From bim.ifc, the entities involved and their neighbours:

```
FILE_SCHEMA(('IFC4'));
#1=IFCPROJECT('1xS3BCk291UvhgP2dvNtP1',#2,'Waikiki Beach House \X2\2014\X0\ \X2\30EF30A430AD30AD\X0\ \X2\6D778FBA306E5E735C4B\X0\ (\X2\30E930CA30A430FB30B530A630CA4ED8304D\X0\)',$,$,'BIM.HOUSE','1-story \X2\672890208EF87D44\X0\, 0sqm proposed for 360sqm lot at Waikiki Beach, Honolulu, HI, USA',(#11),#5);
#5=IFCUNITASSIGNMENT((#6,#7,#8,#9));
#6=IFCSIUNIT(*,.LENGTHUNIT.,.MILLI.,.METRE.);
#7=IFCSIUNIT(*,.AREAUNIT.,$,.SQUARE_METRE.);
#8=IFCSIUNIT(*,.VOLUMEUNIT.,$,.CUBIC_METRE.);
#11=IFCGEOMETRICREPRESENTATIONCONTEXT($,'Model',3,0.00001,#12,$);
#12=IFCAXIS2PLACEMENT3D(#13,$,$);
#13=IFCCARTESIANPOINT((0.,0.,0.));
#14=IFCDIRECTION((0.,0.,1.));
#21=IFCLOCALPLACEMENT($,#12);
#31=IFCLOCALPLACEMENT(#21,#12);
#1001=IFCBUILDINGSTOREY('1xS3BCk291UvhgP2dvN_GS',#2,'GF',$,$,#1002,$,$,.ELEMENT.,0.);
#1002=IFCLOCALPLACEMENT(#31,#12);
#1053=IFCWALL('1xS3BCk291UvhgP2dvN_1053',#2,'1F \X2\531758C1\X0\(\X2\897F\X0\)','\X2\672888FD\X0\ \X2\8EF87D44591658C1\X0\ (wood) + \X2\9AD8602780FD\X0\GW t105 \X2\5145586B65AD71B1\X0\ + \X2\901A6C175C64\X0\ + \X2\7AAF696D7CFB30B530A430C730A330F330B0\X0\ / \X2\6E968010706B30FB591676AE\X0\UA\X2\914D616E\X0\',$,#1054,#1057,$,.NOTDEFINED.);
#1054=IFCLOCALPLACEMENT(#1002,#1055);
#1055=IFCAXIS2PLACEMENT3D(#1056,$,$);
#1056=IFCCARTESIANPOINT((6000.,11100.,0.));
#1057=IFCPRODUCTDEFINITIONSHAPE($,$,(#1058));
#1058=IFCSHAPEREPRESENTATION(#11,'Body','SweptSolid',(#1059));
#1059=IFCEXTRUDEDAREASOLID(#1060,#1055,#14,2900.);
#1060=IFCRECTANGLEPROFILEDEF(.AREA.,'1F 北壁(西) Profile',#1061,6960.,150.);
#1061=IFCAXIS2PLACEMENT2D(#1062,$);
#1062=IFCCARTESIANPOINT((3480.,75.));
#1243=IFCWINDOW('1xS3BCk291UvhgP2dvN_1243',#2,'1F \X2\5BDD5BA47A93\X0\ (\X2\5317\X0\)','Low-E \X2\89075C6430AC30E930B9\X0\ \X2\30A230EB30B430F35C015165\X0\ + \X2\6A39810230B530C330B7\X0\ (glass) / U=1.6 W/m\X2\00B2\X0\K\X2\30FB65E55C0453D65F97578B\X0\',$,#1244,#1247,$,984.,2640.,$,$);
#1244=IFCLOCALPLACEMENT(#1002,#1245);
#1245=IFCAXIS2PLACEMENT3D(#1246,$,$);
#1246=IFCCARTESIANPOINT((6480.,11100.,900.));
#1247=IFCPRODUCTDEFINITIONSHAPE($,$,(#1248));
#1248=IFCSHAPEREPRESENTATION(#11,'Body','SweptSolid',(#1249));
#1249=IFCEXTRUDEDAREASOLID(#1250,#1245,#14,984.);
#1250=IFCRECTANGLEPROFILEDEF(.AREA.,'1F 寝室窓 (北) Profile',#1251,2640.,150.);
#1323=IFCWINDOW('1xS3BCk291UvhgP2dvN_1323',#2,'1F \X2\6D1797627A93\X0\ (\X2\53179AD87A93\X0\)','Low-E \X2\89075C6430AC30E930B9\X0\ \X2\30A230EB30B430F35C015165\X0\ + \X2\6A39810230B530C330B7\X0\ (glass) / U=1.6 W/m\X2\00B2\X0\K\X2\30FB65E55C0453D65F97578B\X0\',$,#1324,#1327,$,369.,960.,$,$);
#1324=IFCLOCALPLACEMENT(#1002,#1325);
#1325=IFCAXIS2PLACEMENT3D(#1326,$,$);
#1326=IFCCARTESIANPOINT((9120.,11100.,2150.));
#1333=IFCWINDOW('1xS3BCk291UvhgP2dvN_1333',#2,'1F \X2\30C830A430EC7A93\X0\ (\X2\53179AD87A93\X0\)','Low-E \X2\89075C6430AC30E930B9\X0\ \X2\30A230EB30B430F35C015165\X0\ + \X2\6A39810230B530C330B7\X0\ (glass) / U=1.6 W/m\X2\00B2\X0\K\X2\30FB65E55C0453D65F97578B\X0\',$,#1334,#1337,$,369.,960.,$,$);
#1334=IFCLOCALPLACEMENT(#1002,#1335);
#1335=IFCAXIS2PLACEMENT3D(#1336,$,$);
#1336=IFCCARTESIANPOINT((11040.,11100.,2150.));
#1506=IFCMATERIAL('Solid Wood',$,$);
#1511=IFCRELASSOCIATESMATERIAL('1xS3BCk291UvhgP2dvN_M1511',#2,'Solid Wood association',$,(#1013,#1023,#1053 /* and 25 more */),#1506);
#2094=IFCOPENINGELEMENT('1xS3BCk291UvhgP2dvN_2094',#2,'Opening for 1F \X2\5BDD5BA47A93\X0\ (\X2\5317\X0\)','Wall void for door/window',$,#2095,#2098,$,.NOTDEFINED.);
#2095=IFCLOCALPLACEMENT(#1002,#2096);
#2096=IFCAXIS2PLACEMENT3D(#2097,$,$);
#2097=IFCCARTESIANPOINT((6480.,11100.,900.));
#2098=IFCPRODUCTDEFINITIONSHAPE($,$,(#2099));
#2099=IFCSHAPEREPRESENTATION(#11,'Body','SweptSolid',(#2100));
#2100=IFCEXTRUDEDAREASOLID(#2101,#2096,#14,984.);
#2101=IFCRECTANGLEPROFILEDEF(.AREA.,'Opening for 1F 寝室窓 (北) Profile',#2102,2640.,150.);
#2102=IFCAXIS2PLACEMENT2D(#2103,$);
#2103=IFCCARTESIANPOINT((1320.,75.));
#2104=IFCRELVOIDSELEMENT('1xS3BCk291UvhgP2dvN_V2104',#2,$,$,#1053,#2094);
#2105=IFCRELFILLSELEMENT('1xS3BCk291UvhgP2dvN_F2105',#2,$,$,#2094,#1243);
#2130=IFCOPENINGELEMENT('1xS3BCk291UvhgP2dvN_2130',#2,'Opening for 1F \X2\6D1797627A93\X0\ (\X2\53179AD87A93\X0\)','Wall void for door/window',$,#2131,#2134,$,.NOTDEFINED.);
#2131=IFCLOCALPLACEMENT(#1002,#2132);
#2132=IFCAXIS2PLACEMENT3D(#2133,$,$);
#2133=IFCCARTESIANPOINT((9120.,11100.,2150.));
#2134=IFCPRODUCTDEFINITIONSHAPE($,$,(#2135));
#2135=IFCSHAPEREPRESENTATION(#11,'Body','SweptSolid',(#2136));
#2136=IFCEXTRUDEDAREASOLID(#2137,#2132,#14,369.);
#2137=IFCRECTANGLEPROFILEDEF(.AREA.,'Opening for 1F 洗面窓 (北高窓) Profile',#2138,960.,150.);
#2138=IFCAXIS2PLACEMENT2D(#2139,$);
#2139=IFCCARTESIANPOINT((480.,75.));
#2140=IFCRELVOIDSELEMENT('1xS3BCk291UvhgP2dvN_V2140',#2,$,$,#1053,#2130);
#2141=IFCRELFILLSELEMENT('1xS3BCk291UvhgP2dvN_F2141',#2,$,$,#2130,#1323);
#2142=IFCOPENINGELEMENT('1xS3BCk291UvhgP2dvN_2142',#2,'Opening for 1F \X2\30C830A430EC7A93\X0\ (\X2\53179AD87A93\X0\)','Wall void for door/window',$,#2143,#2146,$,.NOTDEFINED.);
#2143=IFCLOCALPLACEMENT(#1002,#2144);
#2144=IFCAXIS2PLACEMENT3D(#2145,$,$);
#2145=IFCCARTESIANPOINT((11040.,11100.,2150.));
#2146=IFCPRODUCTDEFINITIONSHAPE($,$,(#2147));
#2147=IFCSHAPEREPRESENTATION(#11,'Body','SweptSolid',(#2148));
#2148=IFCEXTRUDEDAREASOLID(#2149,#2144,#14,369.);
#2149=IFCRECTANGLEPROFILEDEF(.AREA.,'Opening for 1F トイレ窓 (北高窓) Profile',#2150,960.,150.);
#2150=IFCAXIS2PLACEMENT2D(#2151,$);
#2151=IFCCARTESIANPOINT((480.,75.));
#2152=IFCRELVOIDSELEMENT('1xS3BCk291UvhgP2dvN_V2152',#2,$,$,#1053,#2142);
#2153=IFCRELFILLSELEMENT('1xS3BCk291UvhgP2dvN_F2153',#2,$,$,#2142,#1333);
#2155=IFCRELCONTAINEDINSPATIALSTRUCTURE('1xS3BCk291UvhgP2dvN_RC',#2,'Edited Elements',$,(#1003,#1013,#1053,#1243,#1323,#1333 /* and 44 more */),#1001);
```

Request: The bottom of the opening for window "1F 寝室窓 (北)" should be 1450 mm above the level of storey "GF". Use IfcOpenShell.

```python
import numpy as np
import ifcopenshell
import ifcopenshell.api.geometry
import ifcopenshell.geom
import ifcopenshell.util.element
import ifcopenshell.util.placement
import ifcopenshell.util.shape
import ifcopenshell.util.unit

model = ifcopenshell.open("bim.ifc")
unit_scale = ifcopenshell.util.unit.calculate_unit_scale(model)

window = model.by_guid("1xS3BCk291UvhgP2dvN_1243")
opening = window.FillsVoids[0].RelatingOpeningElement
storey = ifcopenshell.util.element.get_container(window, ifc_class="IfcBuildingStorey")
level = ifcopenshell.util.placement.get_local_placement(storey.ObjectPlacement)[2, 3]

# The opening's origin need not be at the sill, so measure its lowest point.
shape = ifcopenshell.geom.create_shape(ifcopenshell.geom.settings(), opening)
bottom = ifcopenshell.util.shape.get_shape_bottom_elevation(shape, shape.geometry) / unit_scale
dz = level + 1.45 / unit_scale - bottom

shift = np.array([0.0, 0.0, dz])
# The window is not placed relative to its opening, so move both.
for product in (opening, window):
    matrix = ifcopenshell.util.placement.get_local_placement(product.ObjectPlacement)
    matrix[:3, 3] += shift
    ifcopenshell.api.geometry.edit_object_placement(model, product=product, matrix=matrix, is_si=False)

print(f"moved by {dz * unit_scale:+.3f} m")

model.write("bim_rev.ifc")
```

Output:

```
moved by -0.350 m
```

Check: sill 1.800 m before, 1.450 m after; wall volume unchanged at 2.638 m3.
